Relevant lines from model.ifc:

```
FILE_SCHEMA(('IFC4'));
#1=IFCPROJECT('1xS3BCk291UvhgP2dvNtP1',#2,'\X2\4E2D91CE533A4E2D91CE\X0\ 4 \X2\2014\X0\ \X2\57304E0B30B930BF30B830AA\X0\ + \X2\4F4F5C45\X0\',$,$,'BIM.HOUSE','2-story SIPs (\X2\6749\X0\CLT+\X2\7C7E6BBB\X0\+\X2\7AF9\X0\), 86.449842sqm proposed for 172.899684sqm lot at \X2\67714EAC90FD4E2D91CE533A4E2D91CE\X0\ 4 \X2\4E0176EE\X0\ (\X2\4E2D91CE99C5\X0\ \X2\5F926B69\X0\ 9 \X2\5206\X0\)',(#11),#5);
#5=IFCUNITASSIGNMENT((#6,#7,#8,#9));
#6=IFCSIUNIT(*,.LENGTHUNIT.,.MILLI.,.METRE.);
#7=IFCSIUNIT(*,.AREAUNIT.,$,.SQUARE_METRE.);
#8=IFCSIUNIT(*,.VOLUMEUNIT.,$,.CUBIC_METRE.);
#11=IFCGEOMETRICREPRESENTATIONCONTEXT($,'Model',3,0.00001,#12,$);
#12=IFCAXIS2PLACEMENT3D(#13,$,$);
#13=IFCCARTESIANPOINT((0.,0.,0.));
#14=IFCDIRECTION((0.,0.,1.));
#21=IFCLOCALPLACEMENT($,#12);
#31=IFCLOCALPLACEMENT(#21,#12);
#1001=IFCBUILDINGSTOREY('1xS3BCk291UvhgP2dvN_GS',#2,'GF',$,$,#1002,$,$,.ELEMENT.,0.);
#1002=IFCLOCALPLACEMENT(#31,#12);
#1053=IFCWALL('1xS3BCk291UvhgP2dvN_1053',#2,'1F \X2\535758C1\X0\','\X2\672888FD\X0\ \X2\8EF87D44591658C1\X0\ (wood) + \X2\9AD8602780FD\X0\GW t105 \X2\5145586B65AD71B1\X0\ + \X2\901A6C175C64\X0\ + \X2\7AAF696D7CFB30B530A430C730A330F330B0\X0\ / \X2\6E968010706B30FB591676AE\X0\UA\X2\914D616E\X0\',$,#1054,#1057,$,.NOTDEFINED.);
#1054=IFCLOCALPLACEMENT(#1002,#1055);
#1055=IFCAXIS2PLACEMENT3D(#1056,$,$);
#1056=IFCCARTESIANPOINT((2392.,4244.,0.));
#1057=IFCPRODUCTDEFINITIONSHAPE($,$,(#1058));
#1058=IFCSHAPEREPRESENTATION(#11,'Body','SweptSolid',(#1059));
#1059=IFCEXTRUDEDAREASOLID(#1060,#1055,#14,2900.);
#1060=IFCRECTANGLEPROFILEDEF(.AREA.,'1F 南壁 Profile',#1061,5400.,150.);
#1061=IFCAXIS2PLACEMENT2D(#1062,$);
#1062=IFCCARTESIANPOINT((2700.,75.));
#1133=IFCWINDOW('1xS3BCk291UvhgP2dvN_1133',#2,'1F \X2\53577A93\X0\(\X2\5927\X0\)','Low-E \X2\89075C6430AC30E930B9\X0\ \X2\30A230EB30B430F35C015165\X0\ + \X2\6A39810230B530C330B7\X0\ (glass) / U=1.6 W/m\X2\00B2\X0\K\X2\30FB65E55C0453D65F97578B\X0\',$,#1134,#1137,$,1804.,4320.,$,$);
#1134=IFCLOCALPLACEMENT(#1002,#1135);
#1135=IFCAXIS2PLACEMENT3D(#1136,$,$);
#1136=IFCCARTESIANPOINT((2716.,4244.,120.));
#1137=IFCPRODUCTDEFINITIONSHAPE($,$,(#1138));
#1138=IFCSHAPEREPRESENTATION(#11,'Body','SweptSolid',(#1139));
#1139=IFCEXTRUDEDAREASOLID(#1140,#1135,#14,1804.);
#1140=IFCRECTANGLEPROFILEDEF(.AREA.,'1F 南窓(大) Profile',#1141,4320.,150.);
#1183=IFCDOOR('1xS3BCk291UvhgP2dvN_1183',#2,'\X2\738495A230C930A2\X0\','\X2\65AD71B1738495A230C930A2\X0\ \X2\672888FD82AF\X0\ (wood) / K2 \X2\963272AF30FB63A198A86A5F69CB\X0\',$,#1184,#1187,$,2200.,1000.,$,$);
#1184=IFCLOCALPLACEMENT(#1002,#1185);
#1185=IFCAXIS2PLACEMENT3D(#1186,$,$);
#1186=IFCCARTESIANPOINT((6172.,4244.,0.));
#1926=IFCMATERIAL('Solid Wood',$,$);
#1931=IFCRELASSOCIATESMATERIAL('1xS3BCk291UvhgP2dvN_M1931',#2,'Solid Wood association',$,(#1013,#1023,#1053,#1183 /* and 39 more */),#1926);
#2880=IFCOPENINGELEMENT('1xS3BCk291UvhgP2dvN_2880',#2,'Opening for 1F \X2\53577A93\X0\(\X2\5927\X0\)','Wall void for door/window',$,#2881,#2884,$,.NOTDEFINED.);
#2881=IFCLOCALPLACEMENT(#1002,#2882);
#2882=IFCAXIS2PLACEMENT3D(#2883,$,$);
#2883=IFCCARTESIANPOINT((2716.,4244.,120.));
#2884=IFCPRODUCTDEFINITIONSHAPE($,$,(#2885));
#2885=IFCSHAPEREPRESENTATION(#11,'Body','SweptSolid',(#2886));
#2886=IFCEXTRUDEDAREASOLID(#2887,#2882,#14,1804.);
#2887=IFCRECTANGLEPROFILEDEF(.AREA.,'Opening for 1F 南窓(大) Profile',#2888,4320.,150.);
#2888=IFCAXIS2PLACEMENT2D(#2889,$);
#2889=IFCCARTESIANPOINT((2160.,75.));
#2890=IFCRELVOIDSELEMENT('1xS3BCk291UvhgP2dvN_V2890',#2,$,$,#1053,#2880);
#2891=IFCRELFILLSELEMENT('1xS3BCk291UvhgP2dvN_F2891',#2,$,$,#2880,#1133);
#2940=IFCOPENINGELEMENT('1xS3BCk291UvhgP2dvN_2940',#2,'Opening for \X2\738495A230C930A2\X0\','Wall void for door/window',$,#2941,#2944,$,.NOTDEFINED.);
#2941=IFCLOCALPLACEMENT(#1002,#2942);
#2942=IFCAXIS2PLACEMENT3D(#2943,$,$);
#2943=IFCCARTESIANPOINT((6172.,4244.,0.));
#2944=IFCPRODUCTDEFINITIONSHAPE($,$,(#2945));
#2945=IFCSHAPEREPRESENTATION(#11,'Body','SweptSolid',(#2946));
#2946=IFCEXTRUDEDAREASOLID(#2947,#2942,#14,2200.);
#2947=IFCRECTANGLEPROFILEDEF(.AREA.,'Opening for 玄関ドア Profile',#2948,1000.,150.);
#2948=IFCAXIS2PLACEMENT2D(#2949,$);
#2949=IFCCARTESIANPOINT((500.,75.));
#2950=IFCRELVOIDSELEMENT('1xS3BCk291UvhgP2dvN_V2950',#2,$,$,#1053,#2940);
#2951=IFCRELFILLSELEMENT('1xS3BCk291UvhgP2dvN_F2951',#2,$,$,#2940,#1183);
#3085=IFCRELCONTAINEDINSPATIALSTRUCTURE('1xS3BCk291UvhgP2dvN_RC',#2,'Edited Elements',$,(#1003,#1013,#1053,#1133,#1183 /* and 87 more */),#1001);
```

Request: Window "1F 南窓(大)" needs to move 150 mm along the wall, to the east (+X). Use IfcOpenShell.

```python
import ifcopenshell
import ifcopenshell.api.geometry
import ifcopenshell.util.placement
import ifcopenshell.util.unit

model = ifcopenshell.open("model.ifc")
unit_scale = ifcopenshell.util.unit.calculate_unit_scale(model)

window = model.by_guid("1xS3BCk291UvhgP2dvN_1133")
opening = window.FillsVoids[0].RelatingOpeningElement
wall = opening.VoidsElements[0].RelatingBuildingElement

wall_matrix = ifcopenshell.util.placement.get_local_placement(wall.ObjectPlacement)
shift = wall_matrix[:3, 0] * 0.15 / unit_scale
before = ifcopenshell.util.placement.get_local_placement(window.ObjectPlacement)[:3, 3].copy()

# The window is not placed relative to its opening, so move both.
for product in (opening, window):
    matrix = ifcopenshell.util.placement.get_local_placement(product.ObjectPlacement)
    matrix[:3, 3] += shift
    ifcopenshell.api.geometry.edit_object_placement(model, product=product, matrix=matrix, is_si=False)

after = ifcopenshell.util.placement.get_local_placement(window.ObjectPlacement)[:3, 3]
print("window moved by", (after - before).round(3) + 0.0)

model.write("model_rev.ifc")
```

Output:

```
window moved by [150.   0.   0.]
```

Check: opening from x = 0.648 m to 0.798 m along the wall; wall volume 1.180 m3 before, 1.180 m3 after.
